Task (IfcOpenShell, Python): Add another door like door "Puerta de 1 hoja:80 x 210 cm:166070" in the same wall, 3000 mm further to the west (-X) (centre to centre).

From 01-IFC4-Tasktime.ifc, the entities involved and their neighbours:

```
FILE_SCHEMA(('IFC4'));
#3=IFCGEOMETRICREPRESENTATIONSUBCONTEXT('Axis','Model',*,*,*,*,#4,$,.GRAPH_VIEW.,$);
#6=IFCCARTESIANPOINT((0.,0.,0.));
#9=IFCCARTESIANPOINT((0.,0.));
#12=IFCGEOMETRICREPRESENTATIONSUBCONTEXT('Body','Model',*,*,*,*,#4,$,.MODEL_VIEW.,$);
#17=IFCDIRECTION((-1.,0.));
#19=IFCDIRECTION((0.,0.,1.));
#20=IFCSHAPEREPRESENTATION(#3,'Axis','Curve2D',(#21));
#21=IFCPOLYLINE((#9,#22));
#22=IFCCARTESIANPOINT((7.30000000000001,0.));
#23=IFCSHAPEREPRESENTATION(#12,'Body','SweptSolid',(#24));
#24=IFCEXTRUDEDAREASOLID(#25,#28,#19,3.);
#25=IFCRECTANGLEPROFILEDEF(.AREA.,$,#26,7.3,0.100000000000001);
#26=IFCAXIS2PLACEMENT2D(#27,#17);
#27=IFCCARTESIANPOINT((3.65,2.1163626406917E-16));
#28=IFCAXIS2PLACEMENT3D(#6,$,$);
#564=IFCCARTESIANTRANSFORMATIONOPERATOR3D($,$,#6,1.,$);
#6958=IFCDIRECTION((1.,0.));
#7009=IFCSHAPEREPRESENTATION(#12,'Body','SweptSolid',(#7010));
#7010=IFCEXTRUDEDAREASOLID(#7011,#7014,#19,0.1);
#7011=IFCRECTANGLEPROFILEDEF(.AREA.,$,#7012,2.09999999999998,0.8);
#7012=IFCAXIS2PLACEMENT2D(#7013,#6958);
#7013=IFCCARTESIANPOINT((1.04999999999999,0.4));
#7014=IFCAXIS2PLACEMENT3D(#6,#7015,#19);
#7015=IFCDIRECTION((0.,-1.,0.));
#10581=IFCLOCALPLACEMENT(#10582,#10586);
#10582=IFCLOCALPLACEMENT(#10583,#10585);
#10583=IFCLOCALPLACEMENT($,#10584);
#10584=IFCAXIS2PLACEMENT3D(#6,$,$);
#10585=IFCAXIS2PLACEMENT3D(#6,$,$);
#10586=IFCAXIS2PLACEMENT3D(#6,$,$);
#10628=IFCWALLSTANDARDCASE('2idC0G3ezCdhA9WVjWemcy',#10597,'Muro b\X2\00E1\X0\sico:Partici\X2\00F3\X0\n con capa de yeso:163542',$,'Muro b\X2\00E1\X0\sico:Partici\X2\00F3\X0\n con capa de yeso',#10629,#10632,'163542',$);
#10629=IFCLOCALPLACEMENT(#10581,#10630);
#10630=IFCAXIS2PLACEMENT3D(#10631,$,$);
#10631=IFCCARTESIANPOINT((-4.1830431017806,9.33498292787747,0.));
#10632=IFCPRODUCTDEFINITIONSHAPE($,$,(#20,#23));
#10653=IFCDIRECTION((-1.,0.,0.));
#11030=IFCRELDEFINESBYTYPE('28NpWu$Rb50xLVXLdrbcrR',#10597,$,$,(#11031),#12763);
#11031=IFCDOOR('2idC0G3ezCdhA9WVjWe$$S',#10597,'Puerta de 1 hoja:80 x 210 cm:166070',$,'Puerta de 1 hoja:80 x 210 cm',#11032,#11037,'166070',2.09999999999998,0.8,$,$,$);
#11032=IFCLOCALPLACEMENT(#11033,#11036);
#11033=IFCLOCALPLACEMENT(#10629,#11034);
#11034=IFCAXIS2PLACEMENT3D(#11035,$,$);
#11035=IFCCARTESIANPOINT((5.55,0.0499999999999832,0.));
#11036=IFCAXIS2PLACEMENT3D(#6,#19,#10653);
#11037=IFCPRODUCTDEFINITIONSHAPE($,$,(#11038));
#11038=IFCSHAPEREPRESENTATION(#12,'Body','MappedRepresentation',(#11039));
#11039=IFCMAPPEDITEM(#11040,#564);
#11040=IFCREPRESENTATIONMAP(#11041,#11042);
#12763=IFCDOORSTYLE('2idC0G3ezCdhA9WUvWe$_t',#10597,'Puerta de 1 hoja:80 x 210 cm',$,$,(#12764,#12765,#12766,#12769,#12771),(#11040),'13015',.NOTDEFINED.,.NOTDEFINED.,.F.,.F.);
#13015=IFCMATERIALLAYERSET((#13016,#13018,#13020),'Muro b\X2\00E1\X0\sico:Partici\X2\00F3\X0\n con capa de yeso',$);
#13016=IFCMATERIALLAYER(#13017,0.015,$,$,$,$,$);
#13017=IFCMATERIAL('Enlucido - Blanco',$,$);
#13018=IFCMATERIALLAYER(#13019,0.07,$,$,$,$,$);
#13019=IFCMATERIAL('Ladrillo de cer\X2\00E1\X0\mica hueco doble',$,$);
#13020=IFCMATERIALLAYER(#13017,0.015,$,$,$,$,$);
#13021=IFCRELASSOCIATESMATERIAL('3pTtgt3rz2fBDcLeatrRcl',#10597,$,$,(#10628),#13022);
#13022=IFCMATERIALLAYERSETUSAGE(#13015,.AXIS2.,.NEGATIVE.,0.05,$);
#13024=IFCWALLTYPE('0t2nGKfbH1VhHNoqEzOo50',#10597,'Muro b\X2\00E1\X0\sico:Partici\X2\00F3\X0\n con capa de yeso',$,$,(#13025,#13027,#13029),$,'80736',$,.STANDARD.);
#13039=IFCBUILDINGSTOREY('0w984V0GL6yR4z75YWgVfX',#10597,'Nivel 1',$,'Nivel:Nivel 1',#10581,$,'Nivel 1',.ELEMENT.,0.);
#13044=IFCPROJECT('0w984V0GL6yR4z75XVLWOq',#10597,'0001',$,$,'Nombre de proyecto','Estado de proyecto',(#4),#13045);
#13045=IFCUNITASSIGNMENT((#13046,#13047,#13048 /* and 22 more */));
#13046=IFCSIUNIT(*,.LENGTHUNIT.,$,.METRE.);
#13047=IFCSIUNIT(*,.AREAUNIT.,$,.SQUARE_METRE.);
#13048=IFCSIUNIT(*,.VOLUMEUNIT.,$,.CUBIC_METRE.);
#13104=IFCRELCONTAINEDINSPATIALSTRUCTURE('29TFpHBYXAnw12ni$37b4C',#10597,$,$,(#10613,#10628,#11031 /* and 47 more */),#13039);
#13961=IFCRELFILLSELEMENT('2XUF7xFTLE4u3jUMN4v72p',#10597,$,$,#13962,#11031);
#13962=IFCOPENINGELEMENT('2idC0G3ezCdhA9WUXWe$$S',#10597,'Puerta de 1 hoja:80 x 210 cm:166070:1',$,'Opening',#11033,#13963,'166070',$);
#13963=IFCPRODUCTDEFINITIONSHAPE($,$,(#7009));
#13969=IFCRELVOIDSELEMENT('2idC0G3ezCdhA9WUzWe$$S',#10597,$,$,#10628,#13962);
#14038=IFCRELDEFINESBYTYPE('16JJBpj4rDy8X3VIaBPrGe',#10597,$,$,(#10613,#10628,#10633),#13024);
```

```python
import ifcopenshell
import ifcopenshell.api.feature
import ifcopenshell.api.geometry
import ifcopenshell.api.root
import ifcopenshell.geom
import ifcopenshell.util.element
import ifcopenshell.util.placement
import ifcopenshell.util.shape

model = ifcopenshell.open("01-IFC4-Tasktime.ifc")
settings = ifcopenshell.geom.settings()


def volume(element):
    """Net volume in cubic metres, openings subtracted."""
    shape = ifcopenshell.geom.create_shape(settings, element)
    return ifcopenshell.util.shape.get_volume(shape.geometry)


def reuse_history(source, copy):
    """copy_class also copies each property set's owner history, people and application; keep the originals."""
    for rel in copy.IsDefinedBy:
        if rel.is_a("IfcRelDefinesByProperties") and (history := rel.RelatingPropertyDefinition.OwnerHistory):
            rel.RelatingPropertyDefinition.OwnerHistory = source.OwnerHistory
            ifcopenshell.util.element.remove_deep2(model, history)


door = model.by_guid("2idC0G3ezCdhA9WVjWe$$S")
opening = door.FillsVoids[0].RelatingOpeningElement
wall = opening.VoidsElements[0].RelatingBuildingElement
before = volume(wall)
shift = ifcopenshell.util.placement.get_local_placement(wall.ObjectPlacement)[:3, 0] * -3.0

# copy_class copies the void relationship, type, container and properties, but no geometry.
new_opening = ifcopenshell.api.root.copy_class(model, product=opening)
new_opening.Representation = ifcopenshell.util.element.copy_deep(
    model, opening.Representation, exclude=["IfcGeometricRepresentationContext", "IfcRepresentationMap"]
)
new_opening.Name = "Puerta de 1 hoja:80 x 210 cm"
new_opening.Tag = None
new_door = ifcopenshell.api.root.copy_class(model, product=door)
new_door.Representation = ifcopenshell.util.element.copy_deep(
    model, door.Representation, exclude=["IfcGeometricRepresentationContext", "IfcRepresentationMap"]
)
new_door.Name = "Puerta de 1 hoja:80 x 210 cm"
new_door.Tag = None
reuse_history(door, new_door)
ifcopenshell.api.feature.add_filling(model, opening=new_opening, element=new_door)

for old, new in ((opening, new_opening), (door, new_door)):
    matrix = ifcopenshell.util.placement.get_local_placement(old.ObjectPlacement)
    matrix[:3, 3] += shift
    ifcopenshell.api.geometry.edit_object_placement(model, product=new, matrix=matrix, is_si=False)

after = volume(wall)

print(f"wall volume {before:.3f} -> {after:.3f} m3")

model.write("01-IFC4-Tasktime_edited.ifc")
```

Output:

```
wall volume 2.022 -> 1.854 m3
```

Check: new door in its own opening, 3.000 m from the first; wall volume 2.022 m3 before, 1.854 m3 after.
